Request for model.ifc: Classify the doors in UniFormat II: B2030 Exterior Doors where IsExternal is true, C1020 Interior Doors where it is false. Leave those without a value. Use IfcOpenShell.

First a look at what the model holds.

```python
import ifcopenshell
import ifcopenshell.util.element

model = ifcopenshell.open("model.ifc")
print(model.schema)
print("classifications:", [c.Name for c in model.by_type("IfcClassification")])
values = [ifcopenshell.util.element.get_pset(e, "Pset_DoorCommon", "IsExternal") for e in model.by_type("IfcDoor")]
for value in (True, False, None):
    print("IsExternal", value, values.count(value))
```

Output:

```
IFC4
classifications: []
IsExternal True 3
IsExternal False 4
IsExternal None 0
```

```python
import ifcopenshell
import ifcopenshell.api.classification
import ifcopenshell.util.element

model = ifcopenshell.open("model.ifc")

system = ifcopenshell.api.classification.add_classification(model, classification="UniFormat II")

doors = model.by_type("IfcDoor")
external = {e: ifcopenshell.util.element.get_pset(e, "Pset_DoorCommon", "IsExternal") for e in doors}
for flag, code, name in ((True, "B2030", "Exterior Doors"), (False, "C1020", "Interior Doors")):
    products = [e for e in doors if external[e] is flag]
    ifcopenshell.api.classification.add_reference(
        model, products=products, classification=system, identification=code, name=name
    )
    print(code, len(products))

model.write("model_edited.ifc")
```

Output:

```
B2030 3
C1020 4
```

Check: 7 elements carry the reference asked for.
